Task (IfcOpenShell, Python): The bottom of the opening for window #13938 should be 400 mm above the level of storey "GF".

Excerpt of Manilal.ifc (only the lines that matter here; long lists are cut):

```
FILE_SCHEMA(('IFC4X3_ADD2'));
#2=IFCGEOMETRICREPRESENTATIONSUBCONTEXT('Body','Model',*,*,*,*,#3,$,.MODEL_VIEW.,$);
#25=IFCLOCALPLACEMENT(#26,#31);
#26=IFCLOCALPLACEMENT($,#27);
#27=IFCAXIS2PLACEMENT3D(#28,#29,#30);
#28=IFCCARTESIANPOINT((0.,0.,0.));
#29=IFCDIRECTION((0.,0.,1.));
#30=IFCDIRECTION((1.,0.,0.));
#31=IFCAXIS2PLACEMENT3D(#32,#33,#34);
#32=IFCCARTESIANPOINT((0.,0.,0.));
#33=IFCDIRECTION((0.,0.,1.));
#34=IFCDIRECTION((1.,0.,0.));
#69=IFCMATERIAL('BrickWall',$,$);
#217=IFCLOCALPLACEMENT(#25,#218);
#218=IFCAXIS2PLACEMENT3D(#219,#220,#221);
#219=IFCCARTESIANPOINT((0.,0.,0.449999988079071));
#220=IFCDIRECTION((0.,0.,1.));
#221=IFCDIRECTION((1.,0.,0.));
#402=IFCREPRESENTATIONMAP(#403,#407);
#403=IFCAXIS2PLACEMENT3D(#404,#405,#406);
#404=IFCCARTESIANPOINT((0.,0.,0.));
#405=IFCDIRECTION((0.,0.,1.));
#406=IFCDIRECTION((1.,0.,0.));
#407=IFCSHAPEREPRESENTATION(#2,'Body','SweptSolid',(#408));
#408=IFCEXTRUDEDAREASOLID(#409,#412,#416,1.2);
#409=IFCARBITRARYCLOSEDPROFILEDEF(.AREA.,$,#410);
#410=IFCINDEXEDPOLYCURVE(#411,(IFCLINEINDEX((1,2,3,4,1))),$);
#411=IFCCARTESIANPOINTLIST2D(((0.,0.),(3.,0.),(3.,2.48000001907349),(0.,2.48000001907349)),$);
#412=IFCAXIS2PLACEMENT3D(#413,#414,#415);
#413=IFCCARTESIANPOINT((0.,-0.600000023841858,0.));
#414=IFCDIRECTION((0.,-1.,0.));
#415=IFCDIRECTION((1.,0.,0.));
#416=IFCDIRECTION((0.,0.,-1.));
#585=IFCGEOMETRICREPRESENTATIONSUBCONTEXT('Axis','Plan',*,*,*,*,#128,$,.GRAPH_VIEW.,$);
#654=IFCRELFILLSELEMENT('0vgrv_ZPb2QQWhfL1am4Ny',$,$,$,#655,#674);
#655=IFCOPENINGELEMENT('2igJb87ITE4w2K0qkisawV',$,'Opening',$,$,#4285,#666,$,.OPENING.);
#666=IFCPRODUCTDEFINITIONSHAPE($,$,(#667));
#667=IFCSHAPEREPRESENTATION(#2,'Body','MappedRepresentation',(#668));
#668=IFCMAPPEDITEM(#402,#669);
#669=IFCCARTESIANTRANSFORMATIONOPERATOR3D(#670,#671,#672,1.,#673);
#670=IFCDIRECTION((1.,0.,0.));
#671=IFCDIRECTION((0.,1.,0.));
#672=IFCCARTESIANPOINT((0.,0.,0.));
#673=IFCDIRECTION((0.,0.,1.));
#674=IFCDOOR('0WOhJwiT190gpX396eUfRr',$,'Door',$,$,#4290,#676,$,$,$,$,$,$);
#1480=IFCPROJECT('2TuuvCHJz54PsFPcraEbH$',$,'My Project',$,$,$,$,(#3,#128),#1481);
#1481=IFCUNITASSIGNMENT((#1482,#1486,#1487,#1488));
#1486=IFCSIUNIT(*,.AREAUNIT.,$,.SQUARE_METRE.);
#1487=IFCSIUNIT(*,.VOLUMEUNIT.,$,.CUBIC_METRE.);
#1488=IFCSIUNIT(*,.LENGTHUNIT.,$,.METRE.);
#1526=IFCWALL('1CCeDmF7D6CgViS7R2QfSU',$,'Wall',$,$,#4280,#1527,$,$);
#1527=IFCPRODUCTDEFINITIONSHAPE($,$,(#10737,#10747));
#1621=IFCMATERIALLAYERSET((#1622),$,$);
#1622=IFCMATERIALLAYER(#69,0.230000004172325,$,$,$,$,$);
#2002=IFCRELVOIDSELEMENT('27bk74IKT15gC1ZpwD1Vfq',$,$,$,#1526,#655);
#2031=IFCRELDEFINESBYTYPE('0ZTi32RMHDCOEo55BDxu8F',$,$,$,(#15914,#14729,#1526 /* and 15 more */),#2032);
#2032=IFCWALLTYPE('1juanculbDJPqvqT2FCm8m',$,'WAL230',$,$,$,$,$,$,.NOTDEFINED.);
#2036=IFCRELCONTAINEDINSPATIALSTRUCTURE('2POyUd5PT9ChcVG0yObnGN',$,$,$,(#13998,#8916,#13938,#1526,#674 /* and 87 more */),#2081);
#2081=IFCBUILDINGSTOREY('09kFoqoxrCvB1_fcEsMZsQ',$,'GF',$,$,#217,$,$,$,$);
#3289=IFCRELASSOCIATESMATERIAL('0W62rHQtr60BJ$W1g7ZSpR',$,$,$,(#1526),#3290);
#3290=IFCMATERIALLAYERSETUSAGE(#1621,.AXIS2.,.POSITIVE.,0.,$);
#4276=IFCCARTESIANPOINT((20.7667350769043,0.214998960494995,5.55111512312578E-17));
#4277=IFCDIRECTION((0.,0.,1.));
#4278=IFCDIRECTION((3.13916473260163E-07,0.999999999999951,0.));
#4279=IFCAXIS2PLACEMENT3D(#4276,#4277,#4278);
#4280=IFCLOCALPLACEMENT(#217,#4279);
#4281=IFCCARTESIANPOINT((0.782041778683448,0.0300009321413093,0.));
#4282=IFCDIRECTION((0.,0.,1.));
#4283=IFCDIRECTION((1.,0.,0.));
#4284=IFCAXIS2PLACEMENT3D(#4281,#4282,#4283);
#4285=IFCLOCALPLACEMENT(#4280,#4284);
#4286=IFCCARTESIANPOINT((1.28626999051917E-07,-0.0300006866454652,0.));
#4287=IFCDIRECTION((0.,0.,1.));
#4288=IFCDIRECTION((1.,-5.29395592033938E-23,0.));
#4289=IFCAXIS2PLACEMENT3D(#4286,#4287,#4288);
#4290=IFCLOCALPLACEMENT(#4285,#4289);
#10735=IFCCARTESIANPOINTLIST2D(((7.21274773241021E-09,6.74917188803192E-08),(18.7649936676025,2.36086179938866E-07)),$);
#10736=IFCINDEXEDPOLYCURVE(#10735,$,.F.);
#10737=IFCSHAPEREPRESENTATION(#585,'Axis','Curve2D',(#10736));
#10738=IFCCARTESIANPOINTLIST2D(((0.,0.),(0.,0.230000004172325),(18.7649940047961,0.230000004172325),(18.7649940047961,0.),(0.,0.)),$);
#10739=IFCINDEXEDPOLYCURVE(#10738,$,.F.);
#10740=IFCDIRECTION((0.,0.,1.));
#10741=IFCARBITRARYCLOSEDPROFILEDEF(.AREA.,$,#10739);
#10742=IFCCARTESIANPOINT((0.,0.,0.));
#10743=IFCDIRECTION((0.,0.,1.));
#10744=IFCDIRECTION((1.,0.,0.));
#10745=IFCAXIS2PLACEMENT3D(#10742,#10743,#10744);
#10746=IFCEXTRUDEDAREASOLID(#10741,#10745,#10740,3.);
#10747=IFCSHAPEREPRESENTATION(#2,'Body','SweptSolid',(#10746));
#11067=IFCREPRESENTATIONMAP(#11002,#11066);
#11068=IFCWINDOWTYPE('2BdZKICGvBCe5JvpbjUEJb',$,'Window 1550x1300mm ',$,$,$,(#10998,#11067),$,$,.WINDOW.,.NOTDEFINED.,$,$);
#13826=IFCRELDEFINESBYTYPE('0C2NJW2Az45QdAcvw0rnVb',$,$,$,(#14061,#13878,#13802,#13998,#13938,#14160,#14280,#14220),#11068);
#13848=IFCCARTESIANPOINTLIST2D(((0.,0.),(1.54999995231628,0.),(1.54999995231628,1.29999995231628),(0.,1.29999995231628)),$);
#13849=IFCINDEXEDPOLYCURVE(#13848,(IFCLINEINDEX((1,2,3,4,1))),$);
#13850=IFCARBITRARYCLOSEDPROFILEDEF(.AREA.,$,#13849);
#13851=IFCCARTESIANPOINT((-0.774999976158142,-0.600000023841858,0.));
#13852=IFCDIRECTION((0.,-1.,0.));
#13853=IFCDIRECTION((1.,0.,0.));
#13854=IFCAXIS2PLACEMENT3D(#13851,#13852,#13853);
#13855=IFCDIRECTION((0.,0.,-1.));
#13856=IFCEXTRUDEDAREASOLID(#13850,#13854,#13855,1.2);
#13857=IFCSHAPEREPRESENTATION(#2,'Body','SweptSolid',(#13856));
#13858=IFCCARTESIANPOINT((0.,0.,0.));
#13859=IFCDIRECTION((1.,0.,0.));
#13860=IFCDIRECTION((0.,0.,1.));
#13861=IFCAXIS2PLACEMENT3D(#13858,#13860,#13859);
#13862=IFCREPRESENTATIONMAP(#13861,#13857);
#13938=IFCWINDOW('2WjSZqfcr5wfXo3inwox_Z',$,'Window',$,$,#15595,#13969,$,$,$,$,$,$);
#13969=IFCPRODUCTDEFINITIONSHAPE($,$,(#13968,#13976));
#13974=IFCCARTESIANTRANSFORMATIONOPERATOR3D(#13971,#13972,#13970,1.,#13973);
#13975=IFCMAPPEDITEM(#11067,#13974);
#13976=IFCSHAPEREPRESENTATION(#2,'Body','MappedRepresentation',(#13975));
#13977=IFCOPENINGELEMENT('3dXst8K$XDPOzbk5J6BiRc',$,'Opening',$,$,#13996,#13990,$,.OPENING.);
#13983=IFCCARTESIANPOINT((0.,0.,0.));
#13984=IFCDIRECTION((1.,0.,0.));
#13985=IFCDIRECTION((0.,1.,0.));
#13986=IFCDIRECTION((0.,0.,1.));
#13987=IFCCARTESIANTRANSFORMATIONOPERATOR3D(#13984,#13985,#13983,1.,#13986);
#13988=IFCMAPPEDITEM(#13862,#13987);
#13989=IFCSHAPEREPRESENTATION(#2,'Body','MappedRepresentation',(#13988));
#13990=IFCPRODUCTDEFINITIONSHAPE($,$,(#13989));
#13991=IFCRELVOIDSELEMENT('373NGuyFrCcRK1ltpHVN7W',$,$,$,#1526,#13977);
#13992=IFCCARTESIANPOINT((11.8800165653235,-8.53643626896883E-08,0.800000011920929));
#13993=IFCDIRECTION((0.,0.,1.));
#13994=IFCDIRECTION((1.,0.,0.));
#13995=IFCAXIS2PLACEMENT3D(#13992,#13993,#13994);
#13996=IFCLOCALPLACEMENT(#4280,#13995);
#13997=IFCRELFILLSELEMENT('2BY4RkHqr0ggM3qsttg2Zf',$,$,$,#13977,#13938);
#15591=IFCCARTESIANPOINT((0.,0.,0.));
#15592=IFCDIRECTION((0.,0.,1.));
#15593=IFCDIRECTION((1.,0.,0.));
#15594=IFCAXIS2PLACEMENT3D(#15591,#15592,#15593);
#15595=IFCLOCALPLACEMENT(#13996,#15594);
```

```python
import numpy as np
import ifcopenshell
import ifcopenshell.api.geometry
import ifcopenshell.geom
import ifcopenshell.util.element
import ifcopenshell.util.placement
import ifcopenshell.util.shape
import ifcopenshell.util.unit

model = ifcopenshell.open("Manilal.ifc")
unit_scale = ifcopenshell.util.unit.calculate_unit_scale(model)

window = model.by_guid("2WjSZqfcr5wfXo3inwox_Z")
opening = window.FillsVoids[0].RelatingOpeningElement
storey = ifcopenshell.util.element.get_container(window, ifc_class="IfcBuildingStorey")
level = ifcopenshell.util.placement.get_local_placement(storey.ObjectPlacement)[2, 3]

# The opening's origin need not be at the sill, so measure its lowest point.
shape = ifcopenshell.geom.create_shape(ifcopenshell.geom.settings(), opening)
bottom = ifcopenshell.util.shape.get_shape_bottom_elevation(shape, shape.geometry) / unit_scale
dz = level + 0.4 / unit_scale - bottom

shift = np.array([0.0, 0.0, dz])
# The window is placed relative to its opening, so it follows when the opening moves.
matrix = ifcopenshell.util.placement.get_local_placement(opening.ObjectPlacement)
matrix[:3, 3] += shift
ifcopenshell.api.geometry.edit_object_placement(
    model, product=opening, matrix=matrix, is_si=False, should_transform_children=True
)

print(f"moved by {dz * unit_scale:+.3f} m")

model.write("Manilal_updated.ifc")
```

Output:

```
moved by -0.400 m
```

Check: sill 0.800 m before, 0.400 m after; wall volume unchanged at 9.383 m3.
